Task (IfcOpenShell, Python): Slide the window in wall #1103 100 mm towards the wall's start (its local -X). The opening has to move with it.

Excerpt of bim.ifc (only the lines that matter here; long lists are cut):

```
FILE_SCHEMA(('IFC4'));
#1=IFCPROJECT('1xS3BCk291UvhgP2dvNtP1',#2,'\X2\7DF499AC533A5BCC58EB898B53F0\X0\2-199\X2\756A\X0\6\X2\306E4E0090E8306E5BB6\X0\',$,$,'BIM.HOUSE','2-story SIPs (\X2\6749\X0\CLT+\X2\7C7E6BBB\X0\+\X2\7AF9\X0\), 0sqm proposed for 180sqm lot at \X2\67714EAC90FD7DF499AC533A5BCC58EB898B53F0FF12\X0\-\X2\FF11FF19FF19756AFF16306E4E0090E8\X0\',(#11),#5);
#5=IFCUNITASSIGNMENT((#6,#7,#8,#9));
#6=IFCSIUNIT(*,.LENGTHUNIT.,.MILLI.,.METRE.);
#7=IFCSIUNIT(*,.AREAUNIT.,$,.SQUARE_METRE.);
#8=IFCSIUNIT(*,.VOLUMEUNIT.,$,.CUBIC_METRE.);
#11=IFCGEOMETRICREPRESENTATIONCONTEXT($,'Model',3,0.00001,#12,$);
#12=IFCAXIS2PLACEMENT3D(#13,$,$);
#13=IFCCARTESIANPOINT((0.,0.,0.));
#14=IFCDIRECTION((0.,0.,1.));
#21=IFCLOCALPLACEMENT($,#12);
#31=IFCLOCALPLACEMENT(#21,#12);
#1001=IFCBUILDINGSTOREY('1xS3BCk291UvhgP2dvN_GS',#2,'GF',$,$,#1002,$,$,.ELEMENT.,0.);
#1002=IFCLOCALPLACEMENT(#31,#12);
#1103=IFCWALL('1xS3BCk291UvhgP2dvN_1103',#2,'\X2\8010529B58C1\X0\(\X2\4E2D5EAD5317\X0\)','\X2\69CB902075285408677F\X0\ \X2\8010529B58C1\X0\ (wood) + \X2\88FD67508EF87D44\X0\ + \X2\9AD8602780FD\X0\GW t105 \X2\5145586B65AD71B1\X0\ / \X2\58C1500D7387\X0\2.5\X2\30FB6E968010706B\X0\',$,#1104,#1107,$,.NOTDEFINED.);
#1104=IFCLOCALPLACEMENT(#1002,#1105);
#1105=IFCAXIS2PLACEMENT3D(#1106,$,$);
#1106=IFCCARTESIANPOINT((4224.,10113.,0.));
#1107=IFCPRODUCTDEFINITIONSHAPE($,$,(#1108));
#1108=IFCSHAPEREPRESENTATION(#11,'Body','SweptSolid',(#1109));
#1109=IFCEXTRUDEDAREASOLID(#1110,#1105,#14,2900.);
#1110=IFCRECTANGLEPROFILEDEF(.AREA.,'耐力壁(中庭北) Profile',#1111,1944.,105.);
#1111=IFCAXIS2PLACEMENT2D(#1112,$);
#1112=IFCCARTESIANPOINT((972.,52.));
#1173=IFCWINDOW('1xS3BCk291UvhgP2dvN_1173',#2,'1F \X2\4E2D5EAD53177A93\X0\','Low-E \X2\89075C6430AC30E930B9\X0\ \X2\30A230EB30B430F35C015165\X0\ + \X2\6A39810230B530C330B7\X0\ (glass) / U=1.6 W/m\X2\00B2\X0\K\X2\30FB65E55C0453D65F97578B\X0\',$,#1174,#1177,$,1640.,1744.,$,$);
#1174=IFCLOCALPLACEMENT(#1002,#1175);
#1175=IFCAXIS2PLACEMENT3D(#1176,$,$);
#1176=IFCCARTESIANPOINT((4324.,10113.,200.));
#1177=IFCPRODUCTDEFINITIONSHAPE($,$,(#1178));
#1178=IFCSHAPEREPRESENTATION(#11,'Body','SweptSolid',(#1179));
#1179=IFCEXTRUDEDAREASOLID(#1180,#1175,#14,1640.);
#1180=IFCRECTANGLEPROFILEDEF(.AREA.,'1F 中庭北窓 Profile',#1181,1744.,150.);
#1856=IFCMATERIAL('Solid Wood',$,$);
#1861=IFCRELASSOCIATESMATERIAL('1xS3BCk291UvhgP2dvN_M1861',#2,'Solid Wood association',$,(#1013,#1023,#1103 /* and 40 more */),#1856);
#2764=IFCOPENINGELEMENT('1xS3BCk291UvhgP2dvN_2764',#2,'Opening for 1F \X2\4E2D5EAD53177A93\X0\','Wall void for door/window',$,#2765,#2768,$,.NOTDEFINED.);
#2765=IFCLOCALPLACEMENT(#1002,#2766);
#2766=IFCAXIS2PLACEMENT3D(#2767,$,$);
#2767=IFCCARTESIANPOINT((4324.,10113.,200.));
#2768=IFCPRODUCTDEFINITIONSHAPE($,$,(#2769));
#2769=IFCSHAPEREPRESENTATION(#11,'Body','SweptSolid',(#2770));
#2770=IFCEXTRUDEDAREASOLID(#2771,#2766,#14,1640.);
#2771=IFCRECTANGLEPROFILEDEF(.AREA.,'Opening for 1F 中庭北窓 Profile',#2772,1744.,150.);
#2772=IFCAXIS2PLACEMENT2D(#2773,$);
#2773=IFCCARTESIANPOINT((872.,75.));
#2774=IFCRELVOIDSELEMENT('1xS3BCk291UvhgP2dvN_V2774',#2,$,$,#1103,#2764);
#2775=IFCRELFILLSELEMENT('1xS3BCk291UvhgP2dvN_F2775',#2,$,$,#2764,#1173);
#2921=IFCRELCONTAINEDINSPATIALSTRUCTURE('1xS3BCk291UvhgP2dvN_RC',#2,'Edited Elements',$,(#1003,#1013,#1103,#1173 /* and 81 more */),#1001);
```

```python
import ifcopenshell
import ifcopenshell.api.geometry
import ifcopenshell.util.placement
import ifcopenshell.util.unit

model = ifcopenshell.open("bim.ifc")
unit_scale = ifcopenshell.util.unit.calculate_unit_scale(model)

window = model.by_guid("1xS3BCk291UvhgP2dvN_1173")
opening = window.FillsVoids[0].RelatingOpeningElement
wall = opening.VoidsElements[0].RelatingBuildingElement

wall_matrix = ifcopenshell.util.placement.get_local_placement(wall.ObjectPlacement)
shift = wall_matrix[:3, 0] * -0.1 / unit_scale
before = ifcopenshell.util.placement.get_local_placement(window.ObjectPlacement)[:3, 3].copy()

# The window is not placed relative to its opening, so move both.
for product in (opening, window):
    matrix = ifcopenshell.util.placement.get_local_placement(product.ObjectPlacement)
    matrix[:3, 3] += shift
    ifcopenshell.api.geometry.edit_object_placement(model, product=product, matrix=matrix, is_si=False)

after = ifcopenshell.util.placement.get_local_placement(window.ObjectPlacement)[:3, 3]
print("window moved by", (after - before).round(3) + 0.0)

model.write("bim_updated.ifc")
```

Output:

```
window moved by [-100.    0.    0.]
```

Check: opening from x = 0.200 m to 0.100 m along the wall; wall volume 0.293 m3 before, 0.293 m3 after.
